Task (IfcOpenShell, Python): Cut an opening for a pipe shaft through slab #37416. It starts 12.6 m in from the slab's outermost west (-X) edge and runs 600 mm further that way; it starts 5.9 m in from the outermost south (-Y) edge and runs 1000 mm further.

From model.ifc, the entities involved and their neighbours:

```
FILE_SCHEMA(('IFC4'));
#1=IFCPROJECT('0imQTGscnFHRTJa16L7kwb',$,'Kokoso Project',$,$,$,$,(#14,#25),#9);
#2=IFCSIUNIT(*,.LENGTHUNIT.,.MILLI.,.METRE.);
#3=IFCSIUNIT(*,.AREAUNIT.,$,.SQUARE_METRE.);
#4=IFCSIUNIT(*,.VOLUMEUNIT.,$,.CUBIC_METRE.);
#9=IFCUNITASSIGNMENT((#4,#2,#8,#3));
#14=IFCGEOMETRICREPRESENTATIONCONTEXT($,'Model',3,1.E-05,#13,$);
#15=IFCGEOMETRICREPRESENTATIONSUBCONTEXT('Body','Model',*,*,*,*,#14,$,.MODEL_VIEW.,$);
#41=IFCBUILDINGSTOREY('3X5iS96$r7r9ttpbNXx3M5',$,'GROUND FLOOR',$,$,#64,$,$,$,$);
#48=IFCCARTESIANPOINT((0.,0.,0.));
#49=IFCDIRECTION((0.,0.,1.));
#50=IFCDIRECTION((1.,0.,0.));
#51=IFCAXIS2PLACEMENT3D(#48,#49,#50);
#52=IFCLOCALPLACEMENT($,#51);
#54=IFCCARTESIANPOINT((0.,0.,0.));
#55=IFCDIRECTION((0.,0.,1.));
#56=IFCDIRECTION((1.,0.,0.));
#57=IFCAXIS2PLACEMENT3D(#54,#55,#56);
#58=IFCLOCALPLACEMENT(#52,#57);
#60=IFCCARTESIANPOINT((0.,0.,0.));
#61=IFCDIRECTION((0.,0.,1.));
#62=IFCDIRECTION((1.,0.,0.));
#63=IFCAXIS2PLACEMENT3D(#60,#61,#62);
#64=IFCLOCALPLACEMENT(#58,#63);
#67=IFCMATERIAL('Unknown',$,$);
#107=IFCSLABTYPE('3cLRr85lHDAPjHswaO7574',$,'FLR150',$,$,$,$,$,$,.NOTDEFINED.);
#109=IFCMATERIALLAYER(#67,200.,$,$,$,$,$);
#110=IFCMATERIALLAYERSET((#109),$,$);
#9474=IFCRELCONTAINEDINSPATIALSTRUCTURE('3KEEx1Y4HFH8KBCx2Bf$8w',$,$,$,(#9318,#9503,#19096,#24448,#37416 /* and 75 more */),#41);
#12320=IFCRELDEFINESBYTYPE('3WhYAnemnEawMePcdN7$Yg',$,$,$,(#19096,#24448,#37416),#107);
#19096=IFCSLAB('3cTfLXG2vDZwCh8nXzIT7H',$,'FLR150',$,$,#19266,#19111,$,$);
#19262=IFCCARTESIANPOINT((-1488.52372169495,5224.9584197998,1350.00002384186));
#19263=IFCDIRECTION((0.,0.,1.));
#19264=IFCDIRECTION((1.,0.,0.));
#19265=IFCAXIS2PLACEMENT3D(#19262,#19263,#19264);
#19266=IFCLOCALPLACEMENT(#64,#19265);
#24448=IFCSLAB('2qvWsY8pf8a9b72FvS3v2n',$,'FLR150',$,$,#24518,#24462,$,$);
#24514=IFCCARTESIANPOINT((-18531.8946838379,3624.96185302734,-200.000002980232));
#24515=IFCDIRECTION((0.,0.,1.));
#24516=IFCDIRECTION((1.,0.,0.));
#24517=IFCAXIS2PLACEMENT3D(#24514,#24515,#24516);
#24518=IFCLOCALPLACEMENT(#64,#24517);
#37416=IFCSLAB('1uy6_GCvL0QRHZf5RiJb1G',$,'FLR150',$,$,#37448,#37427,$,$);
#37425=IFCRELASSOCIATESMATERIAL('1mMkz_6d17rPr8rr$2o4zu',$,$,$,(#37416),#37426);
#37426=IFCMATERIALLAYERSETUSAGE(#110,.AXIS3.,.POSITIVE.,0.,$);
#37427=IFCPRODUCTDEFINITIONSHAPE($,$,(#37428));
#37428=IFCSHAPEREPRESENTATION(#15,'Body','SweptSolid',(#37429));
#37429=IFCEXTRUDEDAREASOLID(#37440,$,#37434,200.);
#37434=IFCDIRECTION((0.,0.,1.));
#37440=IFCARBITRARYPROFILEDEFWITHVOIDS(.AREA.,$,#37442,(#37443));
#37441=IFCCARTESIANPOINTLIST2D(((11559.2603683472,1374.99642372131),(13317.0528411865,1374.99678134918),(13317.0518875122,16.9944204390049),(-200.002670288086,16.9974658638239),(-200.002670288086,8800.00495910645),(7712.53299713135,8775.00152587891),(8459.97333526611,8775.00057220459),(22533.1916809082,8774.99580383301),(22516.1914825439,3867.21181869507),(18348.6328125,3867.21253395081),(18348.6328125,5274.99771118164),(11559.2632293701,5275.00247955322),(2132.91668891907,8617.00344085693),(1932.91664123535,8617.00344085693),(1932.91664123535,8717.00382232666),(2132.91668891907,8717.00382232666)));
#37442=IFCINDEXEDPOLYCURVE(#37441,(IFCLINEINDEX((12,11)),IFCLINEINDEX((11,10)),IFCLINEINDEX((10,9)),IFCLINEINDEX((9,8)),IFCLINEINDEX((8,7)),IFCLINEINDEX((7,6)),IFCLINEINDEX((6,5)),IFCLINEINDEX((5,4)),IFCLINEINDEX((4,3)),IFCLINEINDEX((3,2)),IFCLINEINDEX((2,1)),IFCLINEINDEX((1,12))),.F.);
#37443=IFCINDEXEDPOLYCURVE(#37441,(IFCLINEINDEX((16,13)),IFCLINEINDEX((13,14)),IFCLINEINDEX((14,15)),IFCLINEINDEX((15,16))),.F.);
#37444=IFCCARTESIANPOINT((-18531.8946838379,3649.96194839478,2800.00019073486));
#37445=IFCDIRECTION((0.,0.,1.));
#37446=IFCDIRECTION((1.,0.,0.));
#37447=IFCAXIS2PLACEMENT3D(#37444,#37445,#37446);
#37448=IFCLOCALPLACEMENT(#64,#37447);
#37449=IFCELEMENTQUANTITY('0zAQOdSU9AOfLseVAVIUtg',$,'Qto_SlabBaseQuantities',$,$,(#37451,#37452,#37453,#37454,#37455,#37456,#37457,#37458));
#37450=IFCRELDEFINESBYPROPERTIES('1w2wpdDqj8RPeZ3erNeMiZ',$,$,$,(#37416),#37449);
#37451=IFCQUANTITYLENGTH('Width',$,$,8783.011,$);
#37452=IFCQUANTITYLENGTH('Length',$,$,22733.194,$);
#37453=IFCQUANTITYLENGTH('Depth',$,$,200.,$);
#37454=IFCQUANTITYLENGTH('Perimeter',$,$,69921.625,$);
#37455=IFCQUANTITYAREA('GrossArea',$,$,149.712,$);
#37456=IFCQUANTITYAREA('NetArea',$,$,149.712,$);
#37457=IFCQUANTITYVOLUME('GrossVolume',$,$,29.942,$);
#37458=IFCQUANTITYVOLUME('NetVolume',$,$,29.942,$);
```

```python
import numpy as np
import ifcopenshell
import ifcopenshell.api.feature
import ifcopenshell.api.geometry
import ifcopenshell.api.pset
import ifcopenshell.api.root
import ifcopenshell.geom
import ifcopenshell.util.element
import ifcopenshell.util.placement
import ifcopenshell.util.representation
import ifcopenshell.util.shape
import ifcopenshell.util.unit

model = ifcopenshell.open("model.ifc")
unit_scale = ifcopenshell.util.unit.calculate_unit_scale(model)
area_scale = ifcopenshell.util.unit.calculate_unit_scale(model, "AREAUNIT")
volume_scale = ifcopenshell.util.unit.calculate_unit_scale(model, "VOLUMEUNIT")
settings = ifcopenshell.geom.settings()


def volume(element):
    """Net volume in cubic metres, openings subtracted."""
    shape = ifcopenshell.geom.create_shape(settings, element)
    return ifcopenshell.util.shape.get_volume(shape.geometry)


slab = model.by_guid("1uy6_GCvL0QRHZf5RiJb1G")
before = volume(slab)

# Extent in the slab's own axes, in metres. The edges named are its -X and -Y sides.
slab_shape = ifcopenshell.geom.create_shape(settings, slab)
vertices = ifcopenshell.util.shape.get_vertices(slab_shape.geometry)
x_min, y_min, bottom = vertices.min(axis=0)
top = vertices[:, 2].max()

opening = ifcopenshell.api.root.create_entity(model, ifc_class="IfcOpeningElement", name="Pipe shaft opening", predefined_type="OPENING")
context = ifcopenshell.util.representation.get_context(model, "Model", "Body", "MODEL_VIEW")
width, depth = 0.6, 1
outline = [(0.0, 0.0), (width, 0.0), (width, depth), (0.0, depth), (0.0, 0.0)]
# Overshoot both faces by 50 mm so the cut is clean.
shape = ifcopenshell.api.geometry.add_slab_representation(
    model, context=context, depth=top - bottom + 0.1, polyline=outline
)
ifcopenshell.api.geometry.assign_representation(model, product=opening, representation=shape)

matrix = ifcopenshell.util.placement.get_local_placement(slab.ObjectPlacement)
matrix[:, 3] = matrix @ np.append(np.array([x_min + 12.6, y_min + 5.9, bottom - 0.05]) / unit_scale, 1.0)
ifcopenshell.api.geometry.edit_object_placement(model, product=opening, matrix=matrix, is_si=False)
ifcopenshell.api.feature.add_feature(model, feature=opening, element=slab)

after = volume(slab)

# Update the slab's stored quantities.
qto = model.by_id(ifcopenshell.util.element.get_pset(slab, "Qto_SlabBaseQuantities", should_inherit=False)["id"])
ifcopenshell.api.pset.edit_qto(model, qto=qto, properties={
    "NetArea": after / (top - bottom) / area_scale,
    "NetVolume": after / volume_scale,
})

print(f"slab volume {before:.3f} -> {after:.3f} m3")

model.write("model_v2.ifc")
```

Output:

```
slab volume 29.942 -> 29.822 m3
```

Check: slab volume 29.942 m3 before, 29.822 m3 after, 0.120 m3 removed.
